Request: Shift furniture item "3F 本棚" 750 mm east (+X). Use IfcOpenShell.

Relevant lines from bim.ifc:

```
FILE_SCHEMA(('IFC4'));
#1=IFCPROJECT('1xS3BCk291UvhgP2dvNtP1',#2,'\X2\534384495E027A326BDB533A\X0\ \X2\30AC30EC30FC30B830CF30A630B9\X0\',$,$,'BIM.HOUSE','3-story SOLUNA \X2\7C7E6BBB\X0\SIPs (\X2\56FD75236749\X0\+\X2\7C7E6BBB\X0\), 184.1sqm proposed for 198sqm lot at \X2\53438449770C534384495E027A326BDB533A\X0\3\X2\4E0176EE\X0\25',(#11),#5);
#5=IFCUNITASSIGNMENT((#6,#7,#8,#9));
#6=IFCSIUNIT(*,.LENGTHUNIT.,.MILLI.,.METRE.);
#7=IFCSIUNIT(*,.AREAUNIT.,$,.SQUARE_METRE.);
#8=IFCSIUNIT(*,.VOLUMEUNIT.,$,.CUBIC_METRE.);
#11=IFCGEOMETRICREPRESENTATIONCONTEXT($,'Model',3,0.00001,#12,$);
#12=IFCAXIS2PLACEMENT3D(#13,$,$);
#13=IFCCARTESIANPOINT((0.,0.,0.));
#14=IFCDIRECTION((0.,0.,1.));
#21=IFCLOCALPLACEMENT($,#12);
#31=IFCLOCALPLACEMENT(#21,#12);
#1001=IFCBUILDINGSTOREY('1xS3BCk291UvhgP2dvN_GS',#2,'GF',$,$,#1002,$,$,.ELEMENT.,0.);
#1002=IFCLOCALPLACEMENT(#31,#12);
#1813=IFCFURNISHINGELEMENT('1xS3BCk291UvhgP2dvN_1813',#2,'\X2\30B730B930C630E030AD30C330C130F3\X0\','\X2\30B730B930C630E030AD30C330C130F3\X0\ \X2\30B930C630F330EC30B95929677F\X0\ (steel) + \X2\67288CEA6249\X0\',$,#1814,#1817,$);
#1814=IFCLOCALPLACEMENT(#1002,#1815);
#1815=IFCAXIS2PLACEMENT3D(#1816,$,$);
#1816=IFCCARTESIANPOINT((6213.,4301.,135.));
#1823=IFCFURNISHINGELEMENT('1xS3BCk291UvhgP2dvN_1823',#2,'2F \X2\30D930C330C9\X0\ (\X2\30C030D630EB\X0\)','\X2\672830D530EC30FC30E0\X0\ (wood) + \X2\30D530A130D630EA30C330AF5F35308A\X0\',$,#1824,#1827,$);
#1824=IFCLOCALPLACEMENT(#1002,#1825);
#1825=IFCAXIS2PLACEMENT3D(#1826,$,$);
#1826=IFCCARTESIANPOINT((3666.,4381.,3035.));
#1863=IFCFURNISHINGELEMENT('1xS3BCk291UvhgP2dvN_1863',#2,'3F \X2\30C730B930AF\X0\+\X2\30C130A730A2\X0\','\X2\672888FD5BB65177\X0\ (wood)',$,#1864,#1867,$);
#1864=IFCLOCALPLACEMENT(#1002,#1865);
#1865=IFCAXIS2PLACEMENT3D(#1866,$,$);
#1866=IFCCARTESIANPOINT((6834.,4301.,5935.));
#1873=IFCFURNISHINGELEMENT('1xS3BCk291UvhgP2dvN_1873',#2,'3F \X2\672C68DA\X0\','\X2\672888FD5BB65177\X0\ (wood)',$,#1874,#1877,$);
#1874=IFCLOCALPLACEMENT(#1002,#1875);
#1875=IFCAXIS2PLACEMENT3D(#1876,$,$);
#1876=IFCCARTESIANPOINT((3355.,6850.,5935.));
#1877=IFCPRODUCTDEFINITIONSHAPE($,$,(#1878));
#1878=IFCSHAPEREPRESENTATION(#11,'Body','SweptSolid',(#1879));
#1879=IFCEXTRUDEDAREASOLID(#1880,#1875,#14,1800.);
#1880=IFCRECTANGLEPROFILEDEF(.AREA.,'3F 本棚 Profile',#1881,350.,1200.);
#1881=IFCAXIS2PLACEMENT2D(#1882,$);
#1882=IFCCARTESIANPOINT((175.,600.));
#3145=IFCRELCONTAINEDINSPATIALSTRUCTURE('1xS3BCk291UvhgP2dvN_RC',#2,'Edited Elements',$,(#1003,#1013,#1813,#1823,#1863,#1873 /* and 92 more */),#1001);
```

```python
import ifcopenshell
import ifcopenshell.api.geometry
import ifcopenshell.util.placement
import ifcopenshell.util.unit

model = ifcopenshell.open("bim.ifc")
unit_scale = ifcopenshell.util.unit.calculate_unit_scale(model)

item = model.by_id(1873)
matrix = ifcopenshell.util.placement.get_local_placement(item.ObjectPlacement)
matrix[0, 3] += 0.75 / unit_scale
ifcopenshell.api.geometry.edit_object_placement(model, product=item, matrix=matrix, is_si=False)

print(ifcopenshell.util.placement.get_local_placement(item.ObjectPlacement).round(3) + 0.0)

model.write("bim_rev.ifc")
```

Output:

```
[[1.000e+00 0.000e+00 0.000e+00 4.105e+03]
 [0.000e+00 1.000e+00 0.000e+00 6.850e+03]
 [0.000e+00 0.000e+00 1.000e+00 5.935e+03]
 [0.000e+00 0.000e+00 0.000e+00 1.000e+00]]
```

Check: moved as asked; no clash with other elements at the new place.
